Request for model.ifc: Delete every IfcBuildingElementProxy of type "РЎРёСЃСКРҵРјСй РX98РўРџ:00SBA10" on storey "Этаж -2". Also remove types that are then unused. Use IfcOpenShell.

First a look at what the model holds.

```python
import ifcopenshell
import ifcopenshell.util.element

model = ifcopenshell.open("model.ifc")
print(model.schema)
storey = next(s for s in model.by_type("IfcBuildingStorey") if s.Name == "Этаж -2")
proxies = [e for e in ifcopenshell.util.element.get_decomposition(storey) if e.is_a("IfcBuildingElementProxy")]
seen = {}
for e in proxies:
    element_type = ifcopenshell.util.element.get_type(e)
    name = element_type.Name if element_type not in (None, e) else None
    seen[name] = seen.get(name, 0) + 1
for name, count in sorted(seen.items(), key=str):
    print(count, "x", name)
```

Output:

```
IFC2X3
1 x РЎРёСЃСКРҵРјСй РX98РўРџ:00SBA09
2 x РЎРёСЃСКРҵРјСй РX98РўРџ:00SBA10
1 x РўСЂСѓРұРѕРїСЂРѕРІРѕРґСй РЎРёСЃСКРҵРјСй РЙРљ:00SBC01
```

```python
import ifcopenshell
import ifcopenshell.api.root
import ifcopenshell.util.element

model = ifcopenshell.open("model.ifc")

storey = next(s for s in model.by_type("IfcBuildingStorey") if s.Name == "Этаж -2")
proxies = [e for e in ifcopenshell.util.element.get_decomposition(storey) if e.is_a("IfcBuildingElementProxy")]
targets = [e for e in proxies if (t := ifcopenshell.util.element.get_type(e)) not in (None, e) and t.Name == "РЎРёСЃСКРҵРјСй РX98РўРџ:00SBA10"]
types = {ifcopenshell.util.element.get_type(e) for e in targets} - {None, *targets}

for e in targets:
    ifcopenshell.api.root.remove_product(model, product=e)
print(len(targets), "removed")

unused = [t for t in types if not ifcopenshell.util.element.get_types(t)]
for t in unused:
    ifcopenshell.api.root.remove_product(model, product=t)
print(len(unused), "unused types removed")

model.write("model_rev.ifc")
```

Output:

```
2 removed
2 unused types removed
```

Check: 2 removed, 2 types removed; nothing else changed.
